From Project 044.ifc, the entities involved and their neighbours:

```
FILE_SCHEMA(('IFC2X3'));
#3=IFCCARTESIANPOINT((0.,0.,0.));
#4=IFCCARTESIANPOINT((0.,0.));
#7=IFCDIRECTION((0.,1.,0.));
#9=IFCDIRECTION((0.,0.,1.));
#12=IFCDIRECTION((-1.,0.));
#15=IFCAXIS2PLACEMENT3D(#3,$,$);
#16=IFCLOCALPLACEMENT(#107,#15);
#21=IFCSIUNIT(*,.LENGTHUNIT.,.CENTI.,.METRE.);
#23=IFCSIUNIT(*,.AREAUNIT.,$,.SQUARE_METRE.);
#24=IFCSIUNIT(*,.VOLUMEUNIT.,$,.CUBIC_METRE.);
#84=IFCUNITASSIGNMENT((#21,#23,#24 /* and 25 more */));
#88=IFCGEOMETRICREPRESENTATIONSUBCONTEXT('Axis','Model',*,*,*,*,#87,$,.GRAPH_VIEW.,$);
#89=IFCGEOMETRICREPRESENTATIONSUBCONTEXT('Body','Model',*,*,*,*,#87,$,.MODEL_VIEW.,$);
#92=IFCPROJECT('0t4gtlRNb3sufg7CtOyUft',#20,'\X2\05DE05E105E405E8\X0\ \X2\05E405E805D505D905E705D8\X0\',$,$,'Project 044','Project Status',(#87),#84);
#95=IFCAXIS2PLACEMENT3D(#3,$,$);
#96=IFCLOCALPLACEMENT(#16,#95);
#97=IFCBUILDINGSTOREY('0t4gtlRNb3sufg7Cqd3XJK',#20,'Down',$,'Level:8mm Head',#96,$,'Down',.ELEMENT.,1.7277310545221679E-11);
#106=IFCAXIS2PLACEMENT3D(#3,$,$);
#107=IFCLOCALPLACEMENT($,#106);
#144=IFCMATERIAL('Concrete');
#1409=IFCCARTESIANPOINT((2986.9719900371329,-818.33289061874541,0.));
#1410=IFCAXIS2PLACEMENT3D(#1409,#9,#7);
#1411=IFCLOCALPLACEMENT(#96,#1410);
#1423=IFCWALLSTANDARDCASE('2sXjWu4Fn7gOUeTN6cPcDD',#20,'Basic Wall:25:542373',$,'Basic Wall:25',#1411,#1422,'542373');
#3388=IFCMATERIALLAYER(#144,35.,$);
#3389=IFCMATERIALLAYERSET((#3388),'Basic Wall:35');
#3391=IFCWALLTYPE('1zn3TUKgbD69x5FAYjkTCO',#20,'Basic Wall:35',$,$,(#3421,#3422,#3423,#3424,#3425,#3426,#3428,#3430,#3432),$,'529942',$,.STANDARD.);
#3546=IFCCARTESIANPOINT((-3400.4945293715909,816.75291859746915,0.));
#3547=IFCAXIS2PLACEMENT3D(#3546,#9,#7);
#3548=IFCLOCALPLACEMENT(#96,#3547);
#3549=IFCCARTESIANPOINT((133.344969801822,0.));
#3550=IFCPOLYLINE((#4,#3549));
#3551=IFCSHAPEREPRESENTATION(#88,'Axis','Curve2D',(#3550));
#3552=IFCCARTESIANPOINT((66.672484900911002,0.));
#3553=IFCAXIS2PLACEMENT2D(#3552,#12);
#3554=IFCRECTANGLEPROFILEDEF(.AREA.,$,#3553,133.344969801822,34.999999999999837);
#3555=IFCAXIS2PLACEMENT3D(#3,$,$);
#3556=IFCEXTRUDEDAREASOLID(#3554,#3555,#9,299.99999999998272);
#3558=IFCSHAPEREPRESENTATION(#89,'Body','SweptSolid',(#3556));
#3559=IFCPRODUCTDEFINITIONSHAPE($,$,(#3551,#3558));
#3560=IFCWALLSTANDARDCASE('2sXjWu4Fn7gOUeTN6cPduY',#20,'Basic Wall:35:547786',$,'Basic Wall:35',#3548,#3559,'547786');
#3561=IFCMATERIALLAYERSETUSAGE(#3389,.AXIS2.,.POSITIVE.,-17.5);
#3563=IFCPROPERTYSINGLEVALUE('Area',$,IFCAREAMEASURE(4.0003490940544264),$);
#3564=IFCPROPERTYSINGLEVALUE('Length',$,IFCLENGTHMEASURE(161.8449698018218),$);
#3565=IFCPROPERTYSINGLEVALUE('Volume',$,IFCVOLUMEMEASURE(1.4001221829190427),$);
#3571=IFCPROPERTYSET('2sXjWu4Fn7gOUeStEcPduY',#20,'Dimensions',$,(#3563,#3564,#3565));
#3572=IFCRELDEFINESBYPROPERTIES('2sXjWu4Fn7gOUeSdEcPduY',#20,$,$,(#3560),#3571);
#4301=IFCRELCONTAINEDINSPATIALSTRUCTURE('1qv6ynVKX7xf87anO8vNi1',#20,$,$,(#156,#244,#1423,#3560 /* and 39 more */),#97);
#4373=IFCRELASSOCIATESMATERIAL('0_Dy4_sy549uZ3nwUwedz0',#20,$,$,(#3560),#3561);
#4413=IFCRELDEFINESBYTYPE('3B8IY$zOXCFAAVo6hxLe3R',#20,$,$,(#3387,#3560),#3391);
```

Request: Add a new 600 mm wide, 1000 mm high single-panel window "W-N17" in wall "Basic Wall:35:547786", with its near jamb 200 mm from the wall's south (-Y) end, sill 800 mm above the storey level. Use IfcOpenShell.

```python
import numpy as np
import ifcopenshell
import ifcopenshell.api.feature
import ifcopenshell.api.geometry
import ifcopenshell.api.pset
import ifcopenshell.api.root
import ifcopenshell.api.spatial
import ifcopenshell.api.type
import ifcopenshell.geom
import ifcopenshell.util.element
import ifcopenshell.util.placement
import ifcopenshell.util.representation
import ifcopenshell.util.shape
import ifcopenshell.util.unit

model = ifcopenshell.open("Project 044.ifc")
unit_scale = ifcopenshell.util.unit.calculate_unit_scale(model)
area_scale = ifcopenshell.util.unit.calculate_unit_scale(model, "AREAUNIT")
volume_scale = ifcopenshell.util.unit.calculate_unit_scale(model, "VOLUMEUNIT")
settings = ifcopenshell.geom.settings()


def volume(element):
    """Net volume in cubic metres, openings subtracted."""
    shape = ifcopenshell.geom.create_shape(settings, element)
    return ifcopenshell.util.shape.get_volume(shape.geometry)


wall = model.by_guid("2sXjWu4Fn7gOUeTN6cPduY")
storey = ifcopenshell.util.element.get_container(wall, ifc_class="IfcBuildingStorey")
context = ifcopenshell.util.representation.get_context(model, "Model", "Body", "MODEL_VIEW")
before = volume(wall)

width, height, from_end, sill = 0.6, 1, 0.2, 0.8  # metres

# The wall runs along its own X axis, and the end named is its -X end.
wall_shape = ifcopenshell.geom.create_shape(settings, wall)
x, y, z = ifcopenshell.util.shape.get_vertices(wall_shape.geometry).T
start = x.min() + from_end
face, thickness = float(y.min()), float(y.max() - y.min())
wall_matrix = ifcopenshell.util.placement.get_local_placement(wall.ObjectPlacement)
level = ifcopenshell.util.placement.get_local_placement(storey.ObjectPlacement)[2, 3]


def in_wall(x, y):
    """Placement at x, y metres in the wall's axes, at sill height."""
    matrix = wall_matrix.copy()
    matrix[:, 3] = wall_matrix @ np.array([x / unit_scale, y / unit_scale, 0.0, 1.0])
    matrix[2, 3] = level + sill / unit_scale
    return matrix


# Opening: a box that overshoots both wall faces by 50 mm.
opening = ifcopenshell.api.root.create_entity(model, ifc_class="IfcOpeningElement")
box = ifcopenshell.api.geometry.add_wall_representation(
    model, context=context, length=width, height=height, thickness=thickness + 0.1
)
ifcopenshell.api.geometry.assign_representation(model, product=opening, representation=box)
ifcopenshell.api.geometry.edit_object_placement(model, product=opening, matrix=in_wall(start, face - 0.05), is_si=False)
ifcopenshell.api.feature.add_feature(model, feature=opening, element=wall)

window = ifcopenshell.api.root.create_entity(model, ifc_class="IfcWindow", name="W-N17")
window.OverallWidth, window.OverallHeight = width / unit_scale, height / unit_scale
body = ifcopenshell.api.geometry.add_window_representation(
    model,
    context=context,
    overall_width=window.OverallWidth,
    overall_height=window.OverallHeight,
    partition_type="SINGLE_PANEL",
)
ifcopenshell.api.geometry.assign_representation(model, product=window, representation=body)
ifcopenshell.api.spatial.assign_container(model, products=[window], relating_structure=storey)
fills = ifcopenshell.api.feature.add_filling(model, opening=opening, element=window)
fills.OwnerHistory = window.OwnerHistory  # required in IFC2X3

# IFC2X3 keeps the operation on the window style.
style = ifcopenshell.api.root.create_entity(model, ifc_class="IfcWindowStyle", name="W-N17")
style.OperationType, style.ConstructionType = "SINGLE_PANEL", "NOTDEFINED"
style.ParameterTakesPrecedence = style.Sizeable = False
ifcopenshell.api.type.assign_type(model, related_objects=[window], relating_type=style)

# Centre the window in the wall's thickness.
ifcopenshell.api.geometry.edit_object_placement(model, product=window, matrix=in_wall(start, face), is_si=False)
window_shape = ifcopenshell.geom.create_shape(settings, window)
depth = ifcopenshell.util.shape.get_vertices(window_shape.geometry)[:, 1]
offset = face + thickness / 2 - (depth.min() + depth.max()) / 2
ifcopenshell.api.geometry.edit_object_placement(model, product=window, matrix=in_wall(start, offset), is_si=False)

after = volume(wall)

# Update the wall's stored quantities.
pset = model.by_id(ifcopenshell.util.element.get_pset(wall, "Dimensions", should_inherit=False)["id"])
ifcopenshell.api.pset.edit_pset(model, pset=pset, properties={
    "Area": model.create_entity("IfcAreaMeasure", after / thickness / area_scale),
    "Volume": model.create_entity("IfcVolumeMeasure", after / volume_scale),
})

print(f"wall volume {before:.3f} -> {after:.3f} m3")

model.write("Project 044_edited.ifc")
```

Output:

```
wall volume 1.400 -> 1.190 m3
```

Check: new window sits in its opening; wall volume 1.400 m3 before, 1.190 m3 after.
